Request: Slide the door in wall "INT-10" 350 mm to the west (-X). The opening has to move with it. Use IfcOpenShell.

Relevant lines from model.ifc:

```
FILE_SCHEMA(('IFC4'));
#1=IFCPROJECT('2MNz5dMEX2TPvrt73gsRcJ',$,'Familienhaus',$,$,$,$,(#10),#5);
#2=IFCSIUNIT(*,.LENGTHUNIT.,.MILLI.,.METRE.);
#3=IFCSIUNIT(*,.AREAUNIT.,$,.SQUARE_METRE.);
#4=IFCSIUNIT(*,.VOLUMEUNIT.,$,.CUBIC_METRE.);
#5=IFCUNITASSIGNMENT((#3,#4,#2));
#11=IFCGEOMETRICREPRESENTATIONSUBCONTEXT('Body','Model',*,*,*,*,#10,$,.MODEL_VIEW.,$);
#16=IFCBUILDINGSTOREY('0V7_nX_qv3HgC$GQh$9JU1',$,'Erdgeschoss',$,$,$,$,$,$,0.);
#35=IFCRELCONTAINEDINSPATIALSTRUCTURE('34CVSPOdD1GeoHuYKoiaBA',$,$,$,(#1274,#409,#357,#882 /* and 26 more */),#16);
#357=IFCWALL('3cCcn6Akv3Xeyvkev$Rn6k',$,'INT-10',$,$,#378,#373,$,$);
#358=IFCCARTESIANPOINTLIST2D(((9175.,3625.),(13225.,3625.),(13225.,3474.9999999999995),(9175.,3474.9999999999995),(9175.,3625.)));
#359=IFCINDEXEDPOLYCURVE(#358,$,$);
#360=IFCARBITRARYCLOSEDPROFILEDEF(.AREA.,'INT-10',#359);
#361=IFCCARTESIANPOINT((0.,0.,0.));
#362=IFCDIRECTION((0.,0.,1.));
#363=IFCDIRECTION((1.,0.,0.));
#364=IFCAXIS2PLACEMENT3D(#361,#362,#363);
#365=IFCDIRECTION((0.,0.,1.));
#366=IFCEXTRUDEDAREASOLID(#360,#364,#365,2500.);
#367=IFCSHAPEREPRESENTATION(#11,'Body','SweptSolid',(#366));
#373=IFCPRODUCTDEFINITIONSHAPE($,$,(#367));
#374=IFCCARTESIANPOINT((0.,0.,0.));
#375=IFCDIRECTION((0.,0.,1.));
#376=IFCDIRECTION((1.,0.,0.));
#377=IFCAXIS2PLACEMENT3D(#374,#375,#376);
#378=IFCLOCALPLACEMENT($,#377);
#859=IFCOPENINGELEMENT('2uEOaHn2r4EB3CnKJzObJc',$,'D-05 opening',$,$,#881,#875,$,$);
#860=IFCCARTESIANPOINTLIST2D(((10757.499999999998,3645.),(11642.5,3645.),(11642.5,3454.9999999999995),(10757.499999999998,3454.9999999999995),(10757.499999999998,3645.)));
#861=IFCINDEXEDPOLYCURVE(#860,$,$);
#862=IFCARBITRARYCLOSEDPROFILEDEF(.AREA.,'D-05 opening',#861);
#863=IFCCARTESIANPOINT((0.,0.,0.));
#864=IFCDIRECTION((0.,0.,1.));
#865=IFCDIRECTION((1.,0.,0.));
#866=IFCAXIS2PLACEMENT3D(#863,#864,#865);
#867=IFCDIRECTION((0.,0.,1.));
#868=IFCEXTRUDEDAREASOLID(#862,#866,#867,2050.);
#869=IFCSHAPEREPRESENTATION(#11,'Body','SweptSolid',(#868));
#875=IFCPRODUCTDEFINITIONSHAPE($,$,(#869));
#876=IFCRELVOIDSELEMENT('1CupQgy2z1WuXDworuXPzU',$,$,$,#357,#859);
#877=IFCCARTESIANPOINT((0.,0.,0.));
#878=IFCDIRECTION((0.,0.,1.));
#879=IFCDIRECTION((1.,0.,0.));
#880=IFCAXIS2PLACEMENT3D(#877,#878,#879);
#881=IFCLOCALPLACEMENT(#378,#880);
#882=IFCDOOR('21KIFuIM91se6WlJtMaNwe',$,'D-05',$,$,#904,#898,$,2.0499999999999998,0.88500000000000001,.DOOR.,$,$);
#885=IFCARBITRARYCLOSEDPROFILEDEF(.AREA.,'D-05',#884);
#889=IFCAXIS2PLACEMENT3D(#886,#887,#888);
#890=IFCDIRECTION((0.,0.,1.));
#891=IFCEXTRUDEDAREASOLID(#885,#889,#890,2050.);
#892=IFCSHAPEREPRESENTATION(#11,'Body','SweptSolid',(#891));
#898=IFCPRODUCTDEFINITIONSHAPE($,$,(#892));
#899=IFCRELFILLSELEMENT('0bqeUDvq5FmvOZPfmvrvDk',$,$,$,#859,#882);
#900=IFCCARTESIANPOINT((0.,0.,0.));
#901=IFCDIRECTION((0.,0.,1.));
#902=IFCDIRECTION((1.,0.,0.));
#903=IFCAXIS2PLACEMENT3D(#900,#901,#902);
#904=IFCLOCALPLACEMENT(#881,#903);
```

```python
import ifcopenshell
import ifcopenshell.api.geometry
import ifcopenshell.util.placement
import ifcopenshell.util.unit

model = ifcopenshell.open("model.ifc")
unit_scale = ifcopenshell.util.unit.calculate_unit_scale(model)

door = model.by_guid("21KIFuIM91se6WlJtMaNwe")
opening = door.FillsVoids[0].RelatingOpeningElement
wall = opening.VoidsElements[0].RelatingBuildingElement

wall_matrix = ifcopenshell.util.placement.get_local_placement(wall.ObjectPlacement)
shift = wall_matrix[:3, 0] * -0.35 / unit_scale
before = ifcopenshell.util.placement.get_local_placement(door.ObjectPlacement)[:3, 3].copy()

# The door is placed relative to its opening, so it follows when the opening moves.
matrix = ifcopenshell.util.placement.get_local_placement(opening.ObjectPlacement)
matrix[:3, 3] += shift
ifcopenshell.api.geometry.edit_object_placement(
    model, product=opening, matrix=matrix, is_si=False, should_transform_children=True
)

after = ifcopenshell.util.placement.get_local_placement(door.ObjectPlacement)[:3, 3]
print("door moved by", (after - before).round(3) + 0.0)

model.write("model_v2.ifc")
```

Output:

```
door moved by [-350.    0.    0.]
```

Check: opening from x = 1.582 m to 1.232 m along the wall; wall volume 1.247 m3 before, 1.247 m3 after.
